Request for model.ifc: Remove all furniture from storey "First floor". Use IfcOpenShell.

First a look at what the model holds.

```python
import ifcopenshell
import ifcopenshell.util.element

model = ifcopenshell.open("model.ifc")
print(model.schema)
storey = next(s for s in model.by_type("IfcBuildingStorey") if s.Name == "First floor")
furniture = [e for e in ifcopenshell.util.element.get_decomposition(storey) if e.is_a("IfcFurnishingElement")]
seen = {}
for e in furniture:
    element_type = ifcopenshell.util.element.get_type(e)
    name = element_type.Name if element_type not in (None, e) else None
    seen[name] = seen.get(name, 0) + 1
for name, count in sorted(seen.items(), key=str):
    print(count, "x", name)
```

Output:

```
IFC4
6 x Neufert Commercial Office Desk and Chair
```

```python
import ifcopenshell
import ifcopenshell.api.root
import ifcopenshell.util.element

model = ifcopenshell.open("model.ifc")

storey = next(s for s in model.by_type("IfcBuildingStorey") if s.Name == "First floor")
furniture = [e for e in ifcopenshell.util.element.get_decomposition(storey) if e.is_a("IfcFurnishingElement")]

for e in furniture:
    ifcopenshell.api.root.remove_product(model, product=e)
print(len(furniture), "removed")

model.write("model-out.ifc")
```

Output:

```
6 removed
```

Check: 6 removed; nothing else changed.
